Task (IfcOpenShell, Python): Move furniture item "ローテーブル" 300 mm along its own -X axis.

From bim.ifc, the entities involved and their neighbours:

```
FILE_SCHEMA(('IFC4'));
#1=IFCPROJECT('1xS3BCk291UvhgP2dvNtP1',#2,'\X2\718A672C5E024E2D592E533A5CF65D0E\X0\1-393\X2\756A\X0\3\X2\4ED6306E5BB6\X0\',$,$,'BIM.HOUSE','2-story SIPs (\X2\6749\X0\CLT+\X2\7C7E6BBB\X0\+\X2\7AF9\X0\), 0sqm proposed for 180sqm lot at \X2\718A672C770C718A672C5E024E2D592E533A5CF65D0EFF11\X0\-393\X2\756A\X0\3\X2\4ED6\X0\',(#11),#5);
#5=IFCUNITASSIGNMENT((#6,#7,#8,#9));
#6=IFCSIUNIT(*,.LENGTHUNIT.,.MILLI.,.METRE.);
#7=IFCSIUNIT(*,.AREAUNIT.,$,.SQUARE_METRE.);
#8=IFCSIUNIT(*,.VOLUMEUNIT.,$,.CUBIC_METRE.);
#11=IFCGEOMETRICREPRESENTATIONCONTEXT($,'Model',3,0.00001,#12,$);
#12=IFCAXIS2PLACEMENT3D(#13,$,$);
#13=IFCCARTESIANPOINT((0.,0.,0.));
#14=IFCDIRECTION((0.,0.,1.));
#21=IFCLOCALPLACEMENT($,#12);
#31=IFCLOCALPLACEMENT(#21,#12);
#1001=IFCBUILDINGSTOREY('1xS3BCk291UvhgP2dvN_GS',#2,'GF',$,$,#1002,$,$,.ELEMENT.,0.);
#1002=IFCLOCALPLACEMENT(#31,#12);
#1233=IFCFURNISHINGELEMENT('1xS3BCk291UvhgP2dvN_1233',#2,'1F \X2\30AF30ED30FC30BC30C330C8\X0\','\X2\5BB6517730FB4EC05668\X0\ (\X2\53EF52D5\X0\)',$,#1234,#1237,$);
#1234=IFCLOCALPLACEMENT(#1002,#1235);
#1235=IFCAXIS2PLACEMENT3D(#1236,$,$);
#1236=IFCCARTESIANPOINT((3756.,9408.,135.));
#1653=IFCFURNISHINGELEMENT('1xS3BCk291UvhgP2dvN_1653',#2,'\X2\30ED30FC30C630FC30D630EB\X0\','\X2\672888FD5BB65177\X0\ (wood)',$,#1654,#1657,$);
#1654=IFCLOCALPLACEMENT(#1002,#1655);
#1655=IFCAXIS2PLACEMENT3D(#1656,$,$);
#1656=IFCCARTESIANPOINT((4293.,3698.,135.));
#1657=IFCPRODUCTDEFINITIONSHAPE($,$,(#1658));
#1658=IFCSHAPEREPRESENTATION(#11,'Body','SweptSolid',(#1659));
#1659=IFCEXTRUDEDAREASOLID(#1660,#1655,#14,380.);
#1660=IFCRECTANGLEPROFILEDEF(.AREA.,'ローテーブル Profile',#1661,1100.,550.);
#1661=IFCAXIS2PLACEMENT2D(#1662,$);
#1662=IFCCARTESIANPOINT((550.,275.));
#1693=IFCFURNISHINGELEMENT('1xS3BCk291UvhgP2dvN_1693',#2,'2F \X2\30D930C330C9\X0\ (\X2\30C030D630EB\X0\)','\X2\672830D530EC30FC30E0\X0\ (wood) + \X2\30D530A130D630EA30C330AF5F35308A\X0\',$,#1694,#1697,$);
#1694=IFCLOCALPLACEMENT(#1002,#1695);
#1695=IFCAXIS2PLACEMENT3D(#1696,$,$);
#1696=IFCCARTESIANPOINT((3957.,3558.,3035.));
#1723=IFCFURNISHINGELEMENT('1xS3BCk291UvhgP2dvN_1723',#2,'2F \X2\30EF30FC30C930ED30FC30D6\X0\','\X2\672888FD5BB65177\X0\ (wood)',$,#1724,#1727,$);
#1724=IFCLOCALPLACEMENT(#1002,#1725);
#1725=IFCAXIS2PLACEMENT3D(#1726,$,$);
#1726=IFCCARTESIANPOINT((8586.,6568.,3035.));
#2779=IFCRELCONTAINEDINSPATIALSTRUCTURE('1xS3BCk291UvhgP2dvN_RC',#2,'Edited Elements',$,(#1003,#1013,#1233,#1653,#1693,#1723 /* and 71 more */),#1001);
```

```python
import ifcopenshell
import ifcopenshell.api.geometry
import ifcopenshell.util.placement
import ifcopenshell.util.unit

model = ifcopenshell.open("bim.ifc")
unit_scale = ifcopenshell.util.unit.calculate_unit_scale(model)

item = model.by_guid("1xS3BCk291UvhgP2dvN_1653")
matrix = ifcopenshell.util.placement.get_local_placement(item.ObjectPlacement)
matrix[:3, 3] -= matrix[:3, 0] * 0.3 / unit_scale
ifcopenshell.api.geometry.edit_object_placement(model, product=item, matrix=matrix, is_si=False)

print(ifcopenshell.util.placement.get_local_placement(item.ObjectPlacement).round(3) + 0.0)

model.write("bim_edited.ifc")
```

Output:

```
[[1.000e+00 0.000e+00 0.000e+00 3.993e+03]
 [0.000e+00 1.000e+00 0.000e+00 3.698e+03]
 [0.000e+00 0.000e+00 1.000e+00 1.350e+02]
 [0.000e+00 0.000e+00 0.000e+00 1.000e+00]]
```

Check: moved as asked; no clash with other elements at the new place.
